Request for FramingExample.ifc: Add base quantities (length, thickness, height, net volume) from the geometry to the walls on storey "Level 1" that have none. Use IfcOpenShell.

First a look at what the model holds.

```python
import ifcopenshell
import ifcopenshell.util.element
import ifcopenshell.util.unit

model = ifcopenshell.open("FramingExample.ifc")
print(model.schema)
for unit_type in ("LENGTHUNIT", "AREAUNIT", "VOLUMEUNIT"):
    print(unit_type, ifcopenshell.util.unit.calculate_unit_scale(model, unit_type))
storey = next(s for s in model.by_type("IfcBuildingStorey") if s.Name == "Level 1")
walls = [e for e in ifcopenshell.util.element.get_decomposition(storey) if e.is_a("IfcWall")]
for e in sorted(walls, key=lambda e: e.id()):
    print(e.id(), e.is_a(), e.Name, list(ifcopenshell.util.element.get_psets(e, qtos_only=True)), sep=" | ")
```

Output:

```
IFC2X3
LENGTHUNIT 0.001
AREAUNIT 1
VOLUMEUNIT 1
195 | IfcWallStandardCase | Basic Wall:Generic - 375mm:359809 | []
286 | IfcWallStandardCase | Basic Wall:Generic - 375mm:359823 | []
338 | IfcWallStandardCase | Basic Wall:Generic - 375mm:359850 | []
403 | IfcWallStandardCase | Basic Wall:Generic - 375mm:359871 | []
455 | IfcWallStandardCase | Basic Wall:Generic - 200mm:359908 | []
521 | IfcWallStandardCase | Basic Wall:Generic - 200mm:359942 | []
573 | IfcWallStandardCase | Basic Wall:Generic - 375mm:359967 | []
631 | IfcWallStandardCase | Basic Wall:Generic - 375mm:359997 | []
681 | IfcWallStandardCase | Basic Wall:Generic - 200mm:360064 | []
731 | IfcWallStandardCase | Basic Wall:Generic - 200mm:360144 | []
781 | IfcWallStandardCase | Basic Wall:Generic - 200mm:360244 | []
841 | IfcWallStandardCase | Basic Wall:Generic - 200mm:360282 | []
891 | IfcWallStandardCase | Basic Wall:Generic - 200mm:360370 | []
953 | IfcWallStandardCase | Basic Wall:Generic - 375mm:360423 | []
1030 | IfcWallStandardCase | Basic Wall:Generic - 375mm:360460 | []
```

```python
import ifcopenshell
import ifcopenshell.api.pset
import ifcopenshell.geom
import ifcopenshell.util.element
import ifcopenshell.util.shape
import ifcopenshell.util.unit

model = ifcopenshell.open("FramingExample.ifc")
unit_scale = ifcopenshell.util.unit.calculate_unit_scale(model)
volume_scale = ifcopenshell.util.unit.calculate_unit_scale(model, "VOLUMEUNIT")
settings = ifcopenshell.geom.settings()

storey = next(s for s in model.by_type("IfcBuildingStorey") if s.Name == "Level 1")
walls = [e for e in ifcopenshell.util.element.get_decomposition(storey) if e.is_a("IfcWall")]

for e in sorted(walls, key=lambda e: e.id()):
    if ifcopenshell.util.element.get_psets(e, qtos_only=True, should_inherit=False):
        continue
    # Geometry comes back in metres, in the element's own axes.
    shape = ifcopenshell.geom.create_shape(settings, e)
    values = {
        "Length": ifcopenshell.util.shape.get_x(shape.geometry) / unit_scale,
        "Width": ifcopenshell.util.shape.get_y(shape.geometry) / unit_scale,
        "Height": ifcopenshell.util.shape.get_z(shape.geometry) / unit_scale,
        "NetVolume": ifcopenshell.util.shape.get_volume(shape.geometry) / volume_scale,
    }
    qto = ifcopenshell.api.pset.add_qto(model, product=e, name="BaseQuantities")
    ifcopenshell.api.pset.edit_qto(model, qto=qto, properties=values)
    print(e.id(), {k: round(v, 3) for k, v in values.items()})

model.write("FramingExample_updated.ifc")
```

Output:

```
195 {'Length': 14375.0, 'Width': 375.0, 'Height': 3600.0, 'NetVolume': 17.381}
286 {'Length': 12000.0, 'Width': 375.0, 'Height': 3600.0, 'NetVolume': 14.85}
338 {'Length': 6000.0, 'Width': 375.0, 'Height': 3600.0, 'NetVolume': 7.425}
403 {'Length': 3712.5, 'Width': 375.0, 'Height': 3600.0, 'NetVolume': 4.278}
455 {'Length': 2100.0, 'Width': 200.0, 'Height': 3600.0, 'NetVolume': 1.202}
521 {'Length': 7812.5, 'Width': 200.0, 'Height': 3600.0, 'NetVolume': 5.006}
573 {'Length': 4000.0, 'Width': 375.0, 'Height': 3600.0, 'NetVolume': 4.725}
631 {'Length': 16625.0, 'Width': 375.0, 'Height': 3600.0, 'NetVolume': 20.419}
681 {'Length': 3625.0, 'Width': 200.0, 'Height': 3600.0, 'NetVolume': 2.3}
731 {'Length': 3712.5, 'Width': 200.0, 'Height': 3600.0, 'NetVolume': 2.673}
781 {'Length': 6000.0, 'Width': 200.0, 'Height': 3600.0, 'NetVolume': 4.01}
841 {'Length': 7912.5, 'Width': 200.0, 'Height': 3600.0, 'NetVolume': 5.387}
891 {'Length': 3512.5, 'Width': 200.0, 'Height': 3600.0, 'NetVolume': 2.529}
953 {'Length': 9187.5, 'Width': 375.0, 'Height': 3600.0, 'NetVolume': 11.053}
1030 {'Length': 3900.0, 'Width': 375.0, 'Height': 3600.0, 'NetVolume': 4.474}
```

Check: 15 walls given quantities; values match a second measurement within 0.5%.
